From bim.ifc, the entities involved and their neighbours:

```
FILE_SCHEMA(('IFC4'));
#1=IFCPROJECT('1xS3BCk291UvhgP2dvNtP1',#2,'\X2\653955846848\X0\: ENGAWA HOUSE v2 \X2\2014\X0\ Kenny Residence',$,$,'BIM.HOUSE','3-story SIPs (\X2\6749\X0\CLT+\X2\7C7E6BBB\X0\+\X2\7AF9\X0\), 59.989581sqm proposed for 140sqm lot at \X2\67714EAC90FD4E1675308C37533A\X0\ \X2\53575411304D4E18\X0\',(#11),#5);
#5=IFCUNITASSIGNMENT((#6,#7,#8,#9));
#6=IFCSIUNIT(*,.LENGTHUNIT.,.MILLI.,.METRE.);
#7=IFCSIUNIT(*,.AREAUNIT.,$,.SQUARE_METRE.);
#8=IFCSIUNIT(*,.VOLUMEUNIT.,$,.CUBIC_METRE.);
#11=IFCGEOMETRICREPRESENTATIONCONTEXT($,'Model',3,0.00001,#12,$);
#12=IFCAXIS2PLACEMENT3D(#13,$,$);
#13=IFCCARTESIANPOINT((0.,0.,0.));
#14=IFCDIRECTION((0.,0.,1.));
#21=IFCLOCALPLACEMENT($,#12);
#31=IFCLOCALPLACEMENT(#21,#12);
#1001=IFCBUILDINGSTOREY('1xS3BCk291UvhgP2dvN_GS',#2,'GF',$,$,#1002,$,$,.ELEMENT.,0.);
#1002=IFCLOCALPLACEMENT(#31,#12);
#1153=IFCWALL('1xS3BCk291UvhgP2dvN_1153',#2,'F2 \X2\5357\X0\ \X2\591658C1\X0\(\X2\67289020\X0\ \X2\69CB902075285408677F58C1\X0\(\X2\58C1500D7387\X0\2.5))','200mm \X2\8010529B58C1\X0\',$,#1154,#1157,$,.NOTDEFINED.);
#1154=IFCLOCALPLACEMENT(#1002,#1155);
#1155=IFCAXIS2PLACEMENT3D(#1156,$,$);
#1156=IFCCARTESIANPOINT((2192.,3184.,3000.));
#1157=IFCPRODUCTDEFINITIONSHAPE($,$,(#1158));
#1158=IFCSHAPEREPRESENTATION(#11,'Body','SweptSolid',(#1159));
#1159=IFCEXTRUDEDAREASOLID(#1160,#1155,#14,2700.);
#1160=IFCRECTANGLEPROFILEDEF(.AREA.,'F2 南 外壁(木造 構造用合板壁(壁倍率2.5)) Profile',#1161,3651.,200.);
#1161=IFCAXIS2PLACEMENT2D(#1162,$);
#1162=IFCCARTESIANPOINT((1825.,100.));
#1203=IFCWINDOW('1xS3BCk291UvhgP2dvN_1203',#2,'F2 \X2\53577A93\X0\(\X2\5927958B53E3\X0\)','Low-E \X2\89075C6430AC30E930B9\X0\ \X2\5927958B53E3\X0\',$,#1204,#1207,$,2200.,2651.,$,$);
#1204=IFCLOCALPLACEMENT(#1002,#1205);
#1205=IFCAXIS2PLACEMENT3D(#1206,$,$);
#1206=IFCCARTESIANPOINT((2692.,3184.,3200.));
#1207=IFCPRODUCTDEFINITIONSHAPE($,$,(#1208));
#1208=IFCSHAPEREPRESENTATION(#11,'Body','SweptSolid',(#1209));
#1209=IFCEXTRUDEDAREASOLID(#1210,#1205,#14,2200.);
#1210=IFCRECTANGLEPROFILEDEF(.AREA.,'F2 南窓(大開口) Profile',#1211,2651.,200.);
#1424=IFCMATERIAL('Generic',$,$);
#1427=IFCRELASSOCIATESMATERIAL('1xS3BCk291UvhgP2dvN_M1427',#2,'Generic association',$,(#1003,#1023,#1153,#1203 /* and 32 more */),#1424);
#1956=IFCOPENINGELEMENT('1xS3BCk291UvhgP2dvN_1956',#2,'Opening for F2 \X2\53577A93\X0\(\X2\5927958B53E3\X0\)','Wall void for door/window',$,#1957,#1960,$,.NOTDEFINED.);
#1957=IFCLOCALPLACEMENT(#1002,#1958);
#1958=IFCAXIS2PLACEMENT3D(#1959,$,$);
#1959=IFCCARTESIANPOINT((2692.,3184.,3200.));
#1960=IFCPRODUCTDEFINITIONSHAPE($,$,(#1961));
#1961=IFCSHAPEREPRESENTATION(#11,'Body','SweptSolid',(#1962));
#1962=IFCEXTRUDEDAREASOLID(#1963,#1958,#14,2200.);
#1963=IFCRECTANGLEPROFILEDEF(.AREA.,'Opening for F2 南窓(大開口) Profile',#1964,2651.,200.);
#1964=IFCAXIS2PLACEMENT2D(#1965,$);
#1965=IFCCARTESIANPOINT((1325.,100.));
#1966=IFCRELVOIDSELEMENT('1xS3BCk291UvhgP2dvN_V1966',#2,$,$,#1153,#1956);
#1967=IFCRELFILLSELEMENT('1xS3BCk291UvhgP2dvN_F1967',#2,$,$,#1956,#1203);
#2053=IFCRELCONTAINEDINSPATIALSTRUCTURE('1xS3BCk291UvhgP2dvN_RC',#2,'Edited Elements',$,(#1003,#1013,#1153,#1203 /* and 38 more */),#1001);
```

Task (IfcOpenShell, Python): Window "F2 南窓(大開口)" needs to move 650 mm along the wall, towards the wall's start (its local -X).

```python
import ifcopenshell
import ifcopenshell.api.geometry
import ifcopenshell.util.placement

model = ifcopenshell.open("bim.ifc")

window = model.by_guid("1xS3BCk291UvhgP2dvN_1203")
opening = window.FillsVoids[0].RelatingOpeningElement
wall = opening.VoidsElements[0].RelatingBuildingElement

wall_matrix = ifcopenshell.util.placement.get_local_placement(wall.ObjectPlacement)
shift = wall_matrix[:3, 0] * -650.0
before = ifcopenshell.util.placement.get_local_placement(window.ObjectPlacement)[:3, 3].copy()

# The window is not placed relative to its opening, so move both.
for product in (opening, window):
    matrix = ifcopenshell.util.placement.get_local_placement(product.ObjectPlacement)
    matrix[:3, 3] += shift
    ifcopenshell.api.geometry.edit_object_placement(model, product=product, matrix=matrix, is_si=False)

after = ifcopenshell.util.placement.get_local_placement(window.ObjectPlacement)[:3, 3]
print("window moved by", (after - before).round(3) + 0.0)

model.write("bim_edited.ifc")
```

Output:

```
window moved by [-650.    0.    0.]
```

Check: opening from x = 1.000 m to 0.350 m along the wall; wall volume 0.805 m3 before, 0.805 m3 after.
